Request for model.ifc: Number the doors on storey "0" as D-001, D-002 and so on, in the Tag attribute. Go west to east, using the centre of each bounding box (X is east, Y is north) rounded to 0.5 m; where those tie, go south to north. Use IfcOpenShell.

First a look at what the model holds.

```python
import ifcopenshell
import ifcopenshell.util.element
import ifcopenshell.util.placement

model = ifcopenshell.open("model.ifc")
print(model.schema)
storey = next(s for s in model.by_type("IfcBuildingStorey") if s.Name == "0")
doors = [e for e in ifcopenshell.util.element.get_decomposition(storey) if e.is_a("IfcDoor")]
for e in sorted(doors, key=lambda e: e.id()):
    origin = ifcopenshell.util.placement.get_local_placement(e.ObjectPlacement)[:3, 3]
    print(e.id(), e.Tag, e.Name, origin.round(2) + 0.0, sep=" | ")
```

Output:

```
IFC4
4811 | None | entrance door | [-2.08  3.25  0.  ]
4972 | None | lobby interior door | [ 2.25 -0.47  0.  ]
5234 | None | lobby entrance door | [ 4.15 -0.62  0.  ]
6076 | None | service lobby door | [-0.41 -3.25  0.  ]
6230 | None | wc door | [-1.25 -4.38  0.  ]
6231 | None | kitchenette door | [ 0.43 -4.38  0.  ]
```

```python
import ifcopenshell
import ifcopenshell.geom
import ifcopenshell.util.element
import ifcopenshell.util.shape

model = ifcopenshell.open("model.ifc")
settings = ifcopenshell.geom.settings()
settings.set("use-world-coords", True)


def centre(element):
    shape = ifcopenshell.geom.create_shape(settings, element)
    return ifcopenshell.util.shape.get_bbox_centroid(shape.geometry)


storey = next(s for s in model.by_type("IfcBuildingStorey") if s.Name == "0")
doors = [e for e in ifcopenshell.util.element.get_decomposition(storey) if e.is_a("IfcDoor")]

# Insertion points can sit at a corner or the storey origin, so sort by the geometry (in metres).
centres = {e: centre(e) for e in doors}
doors.sort(key=lambda e: (round(centres[e][0] / 0.5), centres[e][1]))

for i, e in enumerate(doors, start=1):
    number = f"D-0{i:02d}"
    e.Tag = number
    print(e.id(), number)

model.write("model-out.ifc")
```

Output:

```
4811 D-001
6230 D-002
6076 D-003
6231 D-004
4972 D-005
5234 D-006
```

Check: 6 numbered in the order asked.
